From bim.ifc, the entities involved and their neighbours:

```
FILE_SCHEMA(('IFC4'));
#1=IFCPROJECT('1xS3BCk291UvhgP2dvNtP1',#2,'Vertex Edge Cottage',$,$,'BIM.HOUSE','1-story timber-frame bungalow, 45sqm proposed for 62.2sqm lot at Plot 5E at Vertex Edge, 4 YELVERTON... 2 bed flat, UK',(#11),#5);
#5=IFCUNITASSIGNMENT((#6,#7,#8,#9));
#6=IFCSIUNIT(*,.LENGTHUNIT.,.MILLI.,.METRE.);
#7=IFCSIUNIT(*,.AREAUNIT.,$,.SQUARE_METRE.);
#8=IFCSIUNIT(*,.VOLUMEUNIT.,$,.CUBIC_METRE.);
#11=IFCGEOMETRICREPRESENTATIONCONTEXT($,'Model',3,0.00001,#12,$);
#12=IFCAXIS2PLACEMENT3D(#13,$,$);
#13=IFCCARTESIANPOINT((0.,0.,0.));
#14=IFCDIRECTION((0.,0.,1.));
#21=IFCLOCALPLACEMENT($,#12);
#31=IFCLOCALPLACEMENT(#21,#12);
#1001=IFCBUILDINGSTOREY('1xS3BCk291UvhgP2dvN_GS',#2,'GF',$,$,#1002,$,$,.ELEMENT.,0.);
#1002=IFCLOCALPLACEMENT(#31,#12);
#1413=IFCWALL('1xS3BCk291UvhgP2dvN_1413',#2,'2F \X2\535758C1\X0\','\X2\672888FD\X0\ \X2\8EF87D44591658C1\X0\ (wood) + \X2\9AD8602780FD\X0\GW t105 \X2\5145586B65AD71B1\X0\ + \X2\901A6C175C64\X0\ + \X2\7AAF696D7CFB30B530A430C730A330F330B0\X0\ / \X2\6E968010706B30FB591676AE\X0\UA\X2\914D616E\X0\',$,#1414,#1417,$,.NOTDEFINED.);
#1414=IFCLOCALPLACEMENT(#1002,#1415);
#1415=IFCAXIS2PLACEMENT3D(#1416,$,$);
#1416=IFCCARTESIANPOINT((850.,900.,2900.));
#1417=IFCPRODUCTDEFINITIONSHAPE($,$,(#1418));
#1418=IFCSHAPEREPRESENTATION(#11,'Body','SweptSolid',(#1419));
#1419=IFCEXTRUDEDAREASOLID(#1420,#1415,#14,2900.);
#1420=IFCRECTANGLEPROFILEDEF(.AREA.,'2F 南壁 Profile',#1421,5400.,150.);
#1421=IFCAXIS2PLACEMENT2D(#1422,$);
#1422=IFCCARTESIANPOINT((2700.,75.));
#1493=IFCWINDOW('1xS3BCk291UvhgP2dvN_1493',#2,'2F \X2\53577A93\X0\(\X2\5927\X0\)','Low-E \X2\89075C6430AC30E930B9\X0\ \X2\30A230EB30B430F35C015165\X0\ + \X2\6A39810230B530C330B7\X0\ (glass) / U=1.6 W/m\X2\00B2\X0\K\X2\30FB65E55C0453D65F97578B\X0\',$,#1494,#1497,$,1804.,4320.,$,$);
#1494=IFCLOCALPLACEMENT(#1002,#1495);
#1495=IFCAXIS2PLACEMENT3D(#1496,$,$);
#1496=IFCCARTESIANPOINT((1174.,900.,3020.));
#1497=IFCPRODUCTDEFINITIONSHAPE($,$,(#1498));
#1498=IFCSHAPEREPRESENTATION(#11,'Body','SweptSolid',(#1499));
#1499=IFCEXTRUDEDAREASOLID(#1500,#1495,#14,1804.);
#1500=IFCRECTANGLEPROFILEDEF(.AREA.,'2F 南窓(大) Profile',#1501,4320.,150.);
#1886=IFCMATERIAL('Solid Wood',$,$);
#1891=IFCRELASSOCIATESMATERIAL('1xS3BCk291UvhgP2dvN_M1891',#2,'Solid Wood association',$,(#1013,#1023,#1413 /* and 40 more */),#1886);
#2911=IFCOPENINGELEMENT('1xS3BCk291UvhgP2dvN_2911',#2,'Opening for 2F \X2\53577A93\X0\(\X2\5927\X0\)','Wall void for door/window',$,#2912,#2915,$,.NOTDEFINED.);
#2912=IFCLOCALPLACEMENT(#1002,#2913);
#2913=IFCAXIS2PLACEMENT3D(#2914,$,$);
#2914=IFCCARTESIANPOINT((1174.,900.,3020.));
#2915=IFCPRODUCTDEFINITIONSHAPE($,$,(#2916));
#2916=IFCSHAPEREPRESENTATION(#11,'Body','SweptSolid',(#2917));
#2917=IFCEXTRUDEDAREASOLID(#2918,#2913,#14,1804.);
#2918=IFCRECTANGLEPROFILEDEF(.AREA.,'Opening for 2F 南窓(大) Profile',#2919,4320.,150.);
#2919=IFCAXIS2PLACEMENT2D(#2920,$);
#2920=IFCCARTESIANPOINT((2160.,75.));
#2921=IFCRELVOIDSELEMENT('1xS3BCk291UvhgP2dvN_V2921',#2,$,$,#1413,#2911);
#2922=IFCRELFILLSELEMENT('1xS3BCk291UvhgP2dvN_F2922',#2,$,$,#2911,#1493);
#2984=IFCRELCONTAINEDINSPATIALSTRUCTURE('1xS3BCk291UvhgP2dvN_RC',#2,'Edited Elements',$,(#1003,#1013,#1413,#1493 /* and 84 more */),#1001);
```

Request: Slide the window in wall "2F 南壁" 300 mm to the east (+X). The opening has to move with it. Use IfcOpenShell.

```python
import ifcopenshell
import ifcopenshell.api.geometry
import ifcopenshell.util.placement
import ifcopenshell.util.unit

model = ifcopenshell.open("bim.ifc")
unit_scale = ifcopenshell.util.unit.calculate_unit_scale(model)

window = model.by_guid("1xS3BCk291UvhgP2dvN_1493")
opening = window.FillsVoids[0].RelatingOpeningElement
wall = opening.VoidsElements[0].RelatingBuildingElement

wall_matrix = ifcopenshell.util.placement.get_local_placement(wall.ObjectPlacement)
shift = wall_matrix[:3, 0] * 0.3 / unit_scale
before = ifcopenshell.util.placement.get_local_placement(window.ObjectPlacement)[:3, 3].copy()

# The window is not placed relative to its opening, so move both.
for product in (opening, window):
    matrix = ifcopenshell.util.placement.get_local_placement(product.ObjectPlacement)
    matrix[:3, 3] += shift
    ifcopenshell.api.geometry.edit_object_placement(model, product=product, matrix=matrix, is_si=False)

after = ifcopenshell.util.placement.get_local_placement(window.ObjectPlacement)[:3, 3]
print("window moved by", (after - before).round(3) + 0.0)

model.write("bim-out.ifc")
```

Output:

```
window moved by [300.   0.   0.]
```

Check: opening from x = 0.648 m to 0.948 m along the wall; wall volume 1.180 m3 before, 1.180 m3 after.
